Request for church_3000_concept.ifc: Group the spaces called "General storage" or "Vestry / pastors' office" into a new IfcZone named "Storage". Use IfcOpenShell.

First a look at what the model holds.

```python
import ifcopenshell

model = ifcopenshell.open("church_3000_concept.ifc")
print(model.schema)
seen = {}
for space in model.by_type("IfcSpace"):
    seen[space.LongName] = seen.get(space.LongName, 0) + 1
for name, count in sorted(seen.items(), key=str):
    print(count, "x", name)
print("zones:", [z.Name for z in model.by_type("IfcZone")][:20])
```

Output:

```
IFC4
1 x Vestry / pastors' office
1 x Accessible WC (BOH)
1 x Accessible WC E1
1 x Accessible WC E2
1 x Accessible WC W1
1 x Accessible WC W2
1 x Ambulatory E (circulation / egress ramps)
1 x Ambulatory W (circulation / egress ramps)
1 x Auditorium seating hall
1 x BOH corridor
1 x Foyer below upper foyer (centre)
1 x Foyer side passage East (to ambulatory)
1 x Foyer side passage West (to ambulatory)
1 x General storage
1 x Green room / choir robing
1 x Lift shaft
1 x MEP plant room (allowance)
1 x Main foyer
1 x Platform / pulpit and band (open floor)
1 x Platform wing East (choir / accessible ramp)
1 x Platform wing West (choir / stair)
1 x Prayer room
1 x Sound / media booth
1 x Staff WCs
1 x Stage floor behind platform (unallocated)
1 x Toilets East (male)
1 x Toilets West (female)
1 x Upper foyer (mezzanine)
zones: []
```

```python
import ifcopenshell
import ifcopenshell.api.group
import ifcopenshell.api.root

model = ifcopenshell.open("church_3000_concept.ifc")

names = {"General storage", "Vestry / pastors' office"}
spaces = [s for s in model.by_type("IfcSpace") if s.LongName in names]

zone = ifcopenshell.api.root.create_entity(model, ifc_class="IfcZone", name="Storage")
ifcopenshell.api.group.assign_group(model, products=spaces, group=zone)
print(len(spaces), "spaces in", zone.Name)

model.write("church_3000_concept_rev.ifc")
```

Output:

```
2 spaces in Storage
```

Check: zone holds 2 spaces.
